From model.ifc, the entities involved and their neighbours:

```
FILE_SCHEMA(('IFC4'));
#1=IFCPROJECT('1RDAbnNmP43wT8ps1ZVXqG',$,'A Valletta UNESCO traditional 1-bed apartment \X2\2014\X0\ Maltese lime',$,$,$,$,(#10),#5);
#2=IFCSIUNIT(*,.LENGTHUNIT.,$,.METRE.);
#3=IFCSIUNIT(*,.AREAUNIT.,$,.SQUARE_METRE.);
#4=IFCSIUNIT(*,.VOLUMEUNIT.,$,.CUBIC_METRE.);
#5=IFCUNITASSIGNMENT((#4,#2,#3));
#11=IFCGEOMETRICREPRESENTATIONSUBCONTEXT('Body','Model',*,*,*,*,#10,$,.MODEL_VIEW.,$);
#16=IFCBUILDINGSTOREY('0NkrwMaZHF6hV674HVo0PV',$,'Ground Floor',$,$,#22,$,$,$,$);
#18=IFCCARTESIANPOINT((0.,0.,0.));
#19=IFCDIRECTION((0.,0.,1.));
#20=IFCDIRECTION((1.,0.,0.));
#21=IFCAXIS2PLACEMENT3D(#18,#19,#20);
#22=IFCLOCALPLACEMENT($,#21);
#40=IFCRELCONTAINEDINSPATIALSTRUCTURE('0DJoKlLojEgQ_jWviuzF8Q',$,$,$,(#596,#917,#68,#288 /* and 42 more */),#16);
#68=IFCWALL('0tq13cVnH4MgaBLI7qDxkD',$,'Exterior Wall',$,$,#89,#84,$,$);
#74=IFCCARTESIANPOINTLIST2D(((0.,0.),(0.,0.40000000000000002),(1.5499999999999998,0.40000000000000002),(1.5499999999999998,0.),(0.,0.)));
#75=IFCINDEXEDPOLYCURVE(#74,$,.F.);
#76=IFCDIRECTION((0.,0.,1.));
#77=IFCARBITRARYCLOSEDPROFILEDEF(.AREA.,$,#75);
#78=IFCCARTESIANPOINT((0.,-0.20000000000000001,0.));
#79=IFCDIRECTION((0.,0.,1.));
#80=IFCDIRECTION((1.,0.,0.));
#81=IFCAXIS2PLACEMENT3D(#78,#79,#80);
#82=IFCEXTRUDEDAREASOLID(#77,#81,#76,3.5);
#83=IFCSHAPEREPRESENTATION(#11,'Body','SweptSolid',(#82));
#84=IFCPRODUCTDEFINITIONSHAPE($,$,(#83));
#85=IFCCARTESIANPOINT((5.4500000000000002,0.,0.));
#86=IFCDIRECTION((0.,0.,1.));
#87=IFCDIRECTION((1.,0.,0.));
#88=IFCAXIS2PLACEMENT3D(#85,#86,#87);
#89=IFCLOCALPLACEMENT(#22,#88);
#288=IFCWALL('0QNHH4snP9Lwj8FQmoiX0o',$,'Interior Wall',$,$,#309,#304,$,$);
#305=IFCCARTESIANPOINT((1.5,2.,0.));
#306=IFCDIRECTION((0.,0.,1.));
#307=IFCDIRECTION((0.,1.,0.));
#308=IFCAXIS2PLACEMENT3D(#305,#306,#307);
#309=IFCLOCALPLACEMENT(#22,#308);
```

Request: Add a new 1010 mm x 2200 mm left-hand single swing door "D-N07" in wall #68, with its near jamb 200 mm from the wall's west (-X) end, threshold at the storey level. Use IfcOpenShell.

```python
import numpy as np
import ifcopenshell
import ifcopenshell.api.feature
import ifcopenshell.api.geometry
import ifcopenshell.api.root
import ifcopenshell.api.spatial
import ifcopenshell.geom
import ifcopenshell.util.element
import ifcopenshell.util.placement
import ifcopenshell.util.representation
import ifcopenshell.util.shape
import ifcopenshell.util.unit

model = ifcopenshell.open("model.ifc")
unit_scale = ifcopenshell.util.unit.calculate_unit_scale(model)
settings = ifcopenshell.geom.settings()


def volume(element):
    """Net volume in cubic metres, openings subtracted."""
    shape = ifcopenshell.geom.create_shape(settings, element)
    return ifcopenshell.util.shape.get_volume(shape.geometry)


wall = model.by_id(68)
storey = ifcopenshell.util.element.get_container(wall, ifc_class="IfcBuildingStorey")
context = ifcopenshell.util.representation.get_context(model, "Model", "Body", "MODEL_VIEW")
before = volume(wall)

width, height, from_end, sill = 1.01, 2.2, 0.2, 0.0  # metres

# The wall runs along its own X axis, and the end named is its -X end.
wall_shape = ifcopenshell.geom.create_shape(settings, wall)
x, y, z = ifcopenshell.util.shape.get_vertices(wall_shape.geometry).T
start = x.min() + from_end
face, thickness = float(y.min()), float(y.max() - y.min())
wall_matrix = ifcopenshell.util.placement.get_local_placement(wall.ObjectPlacement)
level = ifcopenshell.util.placement.get_local_placement(storey.ObjectPlacement)[2, 3]


def in_wall(x, y):
    """Placement at x, y metres in the wall's axes, at sill height."""
    matrix = wall_matrix.copy()
    matrix[:, 3] = wall_matrix @ np.array([x / unit_scale, y / unit_scale, 0.0, 1.0])
    matrix[2, 3] = level + sill / unit_scale
    return matrix


# Opening: a box that overshoots both wall faces by 50 mm.
opening = ifcopenshell.api.root.create_entity(model, ifc_class="IfcOpeningElement", predefined_type="OPENING")
box = ifcopenshell.api.geometry.add_wall_representation(
    model, context=context, length=width, height=height, thickness=thickness + 0.1
)
ifcopenshell.api.geometry.assign_representation(model, product=opening, representation=box)
ifcopenshell.api.geometry.edit_object_placement(model, product=opening, matrix=in_wall(start, face - 0.05), is_si=False)
ifcopenshell.api.feature.add_feature(model, feature=opening, element=wall)

door = ifcopenshell.api.root.create_entity(model, ifc_class="IfcDoor", name="D-N07", predefined_type="DOOR")
door.OverallWidth, door.OverallHeight = width / unit_scale, height / unit_scale
door.OperationType = "SINGLE_SWING_LEFT"
body = ifcopenshell.api.geometry.add_door_representation(
    model,
    context=context,
    overall_width=door.OverallWidth,
    overall_height=door.OverallHeight,
    operation_type="SINGLE_SWING_LEFT",
    lining_properties={"LiningDepth": thickness / unit_scale, "ThresholdDepth": thickness / unit_scale},
)
ifcopenshell.api.geometry.assign_representation(model, product=door, representation=body)
ifcopenshell.api.spatial.assign_container(model, products=[door], relating_structure=storey)
ifcopenshell.api.feature.add_filling(model, opening=opening, element=door)

# The lining spans the wall, so the door starts at the wall face.
ifcopenshell.api.geometry.edit_object_placement(model, product=door, matrix=in_wall(start, face), is_si=False)

after = volume(wall)

print(f"wall volume {before:.3f} -> {after:.3f} m3")

model.write("model_updated.ifc")
```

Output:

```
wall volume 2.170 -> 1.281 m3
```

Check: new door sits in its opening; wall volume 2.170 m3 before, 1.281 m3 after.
